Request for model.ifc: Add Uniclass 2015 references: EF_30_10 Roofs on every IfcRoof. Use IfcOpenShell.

First a look at what the model holds.

```python
import ifcopenshell

model = ifcopenshell.open("model.ifc")
print(model.schema)
print("classifications:", [c.Name for c in model.by_type("IfcClassification")])
for ifc_class in ("IfcDoor", "IfcRoof", "IfcStair", "IfcWall", "IfcWindow"):
    print(ifc_class, len(model.by_type(ifc_class)))
```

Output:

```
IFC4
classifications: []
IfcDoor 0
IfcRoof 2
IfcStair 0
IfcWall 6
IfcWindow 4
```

```python
import ifcopenshell
import ifcopenshell.api.classification

model = ifcopenshell.open("model.ifc")

system = ifcopenshell.api.classification.add_classification(model, classification="Uniclass 2015")

codes = {
    "IfcRoof": ("EF_30_10", "Roofs"),
}
for ifc_class, (code, name) in codes.items():
    products = model.by_type(ifc_class)
    ifcopenshell.api.classification.add_reference(
        model, products=products, classification=system, identification=code, name=name
    )
    print(code, len(products))

model.write("model_v2.ifc")
```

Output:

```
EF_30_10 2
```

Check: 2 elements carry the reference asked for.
